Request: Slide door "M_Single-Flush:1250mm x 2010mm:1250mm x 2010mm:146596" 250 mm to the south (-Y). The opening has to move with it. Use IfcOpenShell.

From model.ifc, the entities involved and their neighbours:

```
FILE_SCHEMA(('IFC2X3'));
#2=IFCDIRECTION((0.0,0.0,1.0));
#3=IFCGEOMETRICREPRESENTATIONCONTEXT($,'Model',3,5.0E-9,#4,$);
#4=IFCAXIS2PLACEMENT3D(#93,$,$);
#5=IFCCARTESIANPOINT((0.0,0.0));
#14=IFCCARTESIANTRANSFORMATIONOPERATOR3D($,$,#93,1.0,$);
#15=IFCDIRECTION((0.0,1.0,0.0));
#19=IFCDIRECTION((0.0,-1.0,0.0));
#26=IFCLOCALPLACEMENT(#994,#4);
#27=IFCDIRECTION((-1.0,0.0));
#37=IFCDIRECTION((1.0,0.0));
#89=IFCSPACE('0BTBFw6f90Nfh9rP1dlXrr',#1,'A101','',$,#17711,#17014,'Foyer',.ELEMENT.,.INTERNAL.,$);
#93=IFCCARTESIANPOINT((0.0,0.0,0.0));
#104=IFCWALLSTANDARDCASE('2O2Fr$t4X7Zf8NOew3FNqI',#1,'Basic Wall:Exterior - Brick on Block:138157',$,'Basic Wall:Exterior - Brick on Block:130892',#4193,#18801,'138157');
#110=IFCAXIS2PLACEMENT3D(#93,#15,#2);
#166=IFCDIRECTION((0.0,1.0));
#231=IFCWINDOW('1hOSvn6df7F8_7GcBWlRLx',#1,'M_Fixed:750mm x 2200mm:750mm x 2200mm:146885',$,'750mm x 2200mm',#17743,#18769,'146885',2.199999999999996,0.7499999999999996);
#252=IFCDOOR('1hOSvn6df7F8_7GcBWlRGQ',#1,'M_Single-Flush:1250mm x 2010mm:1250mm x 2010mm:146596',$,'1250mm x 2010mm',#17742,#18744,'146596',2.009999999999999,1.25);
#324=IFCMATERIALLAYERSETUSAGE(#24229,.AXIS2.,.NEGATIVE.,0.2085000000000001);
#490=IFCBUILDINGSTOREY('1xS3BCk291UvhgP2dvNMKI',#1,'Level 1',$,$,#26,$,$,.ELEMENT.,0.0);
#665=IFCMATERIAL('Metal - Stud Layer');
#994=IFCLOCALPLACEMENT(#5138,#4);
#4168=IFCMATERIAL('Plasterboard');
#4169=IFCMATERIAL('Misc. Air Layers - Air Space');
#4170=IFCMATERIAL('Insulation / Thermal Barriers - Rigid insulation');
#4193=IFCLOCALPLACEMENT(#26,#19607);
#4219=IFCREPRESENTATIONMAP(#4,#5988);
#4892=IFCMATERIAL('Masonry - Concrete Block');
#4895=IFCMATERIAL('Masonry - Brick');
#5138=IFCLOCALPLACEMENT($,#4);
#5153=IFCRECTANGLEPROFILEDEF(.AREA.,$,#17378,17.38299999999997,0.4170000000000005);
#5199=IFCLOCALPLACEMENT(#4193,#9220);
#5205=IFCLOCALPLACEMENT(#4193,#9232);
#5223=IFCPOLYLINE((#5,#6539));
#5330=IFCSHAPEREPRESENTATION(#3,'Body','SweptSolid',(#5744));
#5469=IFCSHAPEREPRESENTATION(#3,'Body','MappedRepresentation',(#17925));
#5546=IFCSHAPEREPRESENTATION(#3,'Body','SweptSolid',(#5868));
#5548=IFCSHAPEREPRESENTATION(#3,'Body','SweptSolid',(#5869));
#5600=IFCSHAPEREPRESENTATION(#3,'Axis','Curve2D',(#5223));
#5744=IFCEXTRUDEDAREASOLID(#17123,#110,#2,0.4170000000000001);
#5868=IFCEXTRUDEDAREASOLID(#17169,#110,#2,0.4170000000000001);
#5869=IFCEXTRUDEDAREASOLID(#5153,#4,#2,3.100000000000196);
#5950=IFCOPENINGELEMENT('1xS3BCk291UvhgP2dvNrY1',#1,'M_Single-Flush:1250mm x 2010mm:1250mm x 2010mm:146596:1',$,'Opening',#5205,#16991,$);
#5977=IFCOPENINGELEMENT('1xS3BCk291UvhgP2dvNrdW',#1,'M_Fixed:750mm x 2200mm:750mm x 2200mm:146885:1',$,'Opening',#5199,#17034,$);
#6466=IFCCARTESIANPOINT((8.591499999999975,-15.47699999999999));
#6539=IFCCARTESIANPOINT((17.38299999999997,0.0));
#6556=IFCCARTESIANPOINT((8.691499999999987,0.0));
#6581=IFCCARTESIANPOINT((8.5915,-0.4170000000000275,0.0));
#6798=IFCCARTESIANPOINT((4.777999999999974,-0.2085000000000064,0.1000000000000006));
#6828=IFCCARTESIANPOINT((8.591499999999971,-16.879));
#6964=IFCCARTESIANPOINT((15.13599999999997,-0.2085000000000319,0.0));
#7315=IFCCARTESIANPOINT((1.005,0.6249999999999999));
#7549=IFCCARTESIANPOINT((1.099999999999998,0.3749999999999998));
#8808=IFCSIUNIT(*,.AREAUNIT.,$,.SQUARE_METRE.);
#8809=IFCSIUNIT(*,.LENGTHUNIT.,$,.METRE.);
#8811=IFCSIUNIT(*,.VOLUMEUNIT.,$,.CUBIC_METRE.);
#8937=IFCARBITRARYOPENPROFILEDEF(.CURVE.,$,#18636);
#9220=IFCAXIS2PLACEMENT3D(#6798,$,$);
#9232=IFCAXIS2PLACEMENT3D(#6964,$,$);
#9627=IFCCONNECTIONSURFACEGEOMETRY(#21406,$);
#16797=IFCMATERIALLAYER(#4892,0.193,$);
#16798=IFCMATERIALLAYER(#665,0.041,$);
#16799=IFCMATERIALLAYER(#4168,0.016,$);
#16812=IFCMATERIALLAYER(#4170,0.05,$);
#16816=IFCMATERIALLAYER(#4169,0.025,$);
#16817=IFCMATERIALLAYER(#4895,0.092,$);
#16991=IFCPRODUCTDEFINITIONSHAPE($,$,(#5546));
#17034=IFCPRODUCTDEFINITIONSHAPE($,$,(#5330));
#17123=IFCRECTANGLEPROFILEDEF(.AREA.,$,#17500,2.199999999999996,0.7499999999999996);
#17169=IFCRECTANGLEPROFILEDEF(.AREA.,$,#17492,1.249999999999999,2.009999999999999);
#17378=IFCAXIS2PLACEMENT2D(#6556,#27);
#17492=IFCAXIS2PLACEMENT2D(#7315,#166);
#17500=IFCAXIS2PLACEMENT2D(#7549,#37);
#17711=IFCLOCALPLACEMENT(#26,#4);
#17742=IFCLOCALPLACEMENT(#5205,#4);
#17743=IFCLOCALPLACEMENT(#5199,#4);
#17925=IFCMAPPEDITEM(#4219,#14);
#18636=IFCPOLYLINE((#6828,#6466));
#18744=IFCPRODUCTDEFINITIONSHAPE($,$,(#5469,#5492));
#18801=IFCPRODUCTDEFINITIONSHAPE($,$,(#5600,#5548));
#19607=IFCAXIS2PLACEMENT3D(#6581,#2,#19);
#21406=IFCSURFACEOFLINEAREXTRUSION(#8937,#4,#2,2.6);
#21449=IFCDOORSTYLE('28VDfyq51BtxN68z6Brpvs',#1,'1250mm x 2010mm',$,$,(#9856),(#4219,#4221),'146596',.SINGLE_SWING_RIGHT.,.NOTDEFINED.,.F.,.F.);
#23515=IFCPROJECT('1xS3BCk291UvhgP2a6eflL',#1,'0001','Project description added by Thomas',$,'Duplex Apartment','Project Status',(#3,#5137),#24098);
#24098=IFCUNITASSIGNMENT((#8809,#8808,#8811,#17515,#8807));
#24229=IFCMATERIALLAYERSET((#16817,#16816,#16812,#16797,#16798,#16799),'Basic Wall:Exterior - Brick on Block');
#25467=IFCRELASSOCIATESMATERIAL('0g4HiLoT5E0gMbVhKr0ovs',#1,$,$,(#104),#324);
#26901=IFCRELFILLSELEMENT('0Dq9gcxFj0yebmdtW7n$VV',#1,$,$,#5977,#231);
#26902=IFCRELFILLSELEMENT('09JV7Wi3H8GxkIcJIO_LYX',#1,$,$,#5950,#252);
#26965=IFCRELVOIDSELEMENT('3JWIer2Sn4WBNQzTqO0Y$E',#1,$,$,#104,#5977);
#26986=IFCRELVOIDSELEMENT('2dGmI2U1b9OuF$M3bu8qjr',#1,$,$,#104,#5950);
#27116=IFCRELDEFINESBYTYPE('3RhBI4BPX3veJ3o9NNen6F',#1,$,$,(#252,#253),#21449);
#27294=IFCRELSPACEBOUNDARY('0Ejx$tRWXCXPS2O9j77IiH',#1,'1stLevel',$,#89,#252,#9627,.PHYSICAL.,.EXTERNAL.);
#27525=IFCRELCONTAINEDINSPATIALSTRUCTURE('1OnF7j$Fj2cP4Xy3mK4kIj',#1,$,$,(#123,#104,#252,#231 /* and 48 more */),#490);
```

```python
import numpy as np
import ifcopenshell
import ifcopenshell.api.geometry
import ifcopenshell.util.placement
import ifcopenshell.util.unit

model = ifcopenshell.open("model.ifc")
unit_scale = ifcopenshell.util.unit.calculate_unit_scale(model)

door = model.by_guid("1hOSvn6df7F8_7GcBWlRGQ")
opening = door.FillsVoids[0].RelatingOpeningElement
wall = opening.VoidsElements[0].RelatingBuildingElement

wall_matrix = ifcopenshell.util.placement.get_local_placement(wall.ObjectPlacement)
shift = wall_matrix[:3, 0] * 0.25 / unit_scale
before = ifcopenshell.util.placement.get_local_placement(door.ObjectPlacement)[:3, 3].copy()

# The door is placed relative to its opening, so it follows when the opening moves.
matrix = ifcopenshell.util.placement.get_local_placement(opening.ObjectPlacement)
matrix[:3, 3] += shift
ifcopenshell.api.geometry.edit_object_placement(
    model, product=opening, matrix=matrix, is_si=False, should_transform_children=True
)

# Space boundary surfaces are stored in each space's coordinates; move them too.
for rel in door.ProvidesBoundaries:
    if not rel.ConnectionGeometry:
        continue
    surface = rel.ConnectionGeometry.SurfaceOnRelatingElement
    space_matrix = ifcopenshell.util.placement.get_local_placement(rel.RelatingSpace.ObjectPlacement)
    point = np.array(surface.Position.Location.Coordinates) + space_matrix[:3, :3].T @ shift
    surface.Position = model.createIfcAxis2Placement3D(
        model.createIfcCartesianPoint(point.tolist()), surface.Position.Axis, surface.Position.RefDirection
    )

after = ifcopenshell.util.placement.get_local_placement(door.ObjectPlacement)[:3, 3]
print("door moved by", (after - before).round(3) + 0.0)

model.write("model_rev.ifc")
```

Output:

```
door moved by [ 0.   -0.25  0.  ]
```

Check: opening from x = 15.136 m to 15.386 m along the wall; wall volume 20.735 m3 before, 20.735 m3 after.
